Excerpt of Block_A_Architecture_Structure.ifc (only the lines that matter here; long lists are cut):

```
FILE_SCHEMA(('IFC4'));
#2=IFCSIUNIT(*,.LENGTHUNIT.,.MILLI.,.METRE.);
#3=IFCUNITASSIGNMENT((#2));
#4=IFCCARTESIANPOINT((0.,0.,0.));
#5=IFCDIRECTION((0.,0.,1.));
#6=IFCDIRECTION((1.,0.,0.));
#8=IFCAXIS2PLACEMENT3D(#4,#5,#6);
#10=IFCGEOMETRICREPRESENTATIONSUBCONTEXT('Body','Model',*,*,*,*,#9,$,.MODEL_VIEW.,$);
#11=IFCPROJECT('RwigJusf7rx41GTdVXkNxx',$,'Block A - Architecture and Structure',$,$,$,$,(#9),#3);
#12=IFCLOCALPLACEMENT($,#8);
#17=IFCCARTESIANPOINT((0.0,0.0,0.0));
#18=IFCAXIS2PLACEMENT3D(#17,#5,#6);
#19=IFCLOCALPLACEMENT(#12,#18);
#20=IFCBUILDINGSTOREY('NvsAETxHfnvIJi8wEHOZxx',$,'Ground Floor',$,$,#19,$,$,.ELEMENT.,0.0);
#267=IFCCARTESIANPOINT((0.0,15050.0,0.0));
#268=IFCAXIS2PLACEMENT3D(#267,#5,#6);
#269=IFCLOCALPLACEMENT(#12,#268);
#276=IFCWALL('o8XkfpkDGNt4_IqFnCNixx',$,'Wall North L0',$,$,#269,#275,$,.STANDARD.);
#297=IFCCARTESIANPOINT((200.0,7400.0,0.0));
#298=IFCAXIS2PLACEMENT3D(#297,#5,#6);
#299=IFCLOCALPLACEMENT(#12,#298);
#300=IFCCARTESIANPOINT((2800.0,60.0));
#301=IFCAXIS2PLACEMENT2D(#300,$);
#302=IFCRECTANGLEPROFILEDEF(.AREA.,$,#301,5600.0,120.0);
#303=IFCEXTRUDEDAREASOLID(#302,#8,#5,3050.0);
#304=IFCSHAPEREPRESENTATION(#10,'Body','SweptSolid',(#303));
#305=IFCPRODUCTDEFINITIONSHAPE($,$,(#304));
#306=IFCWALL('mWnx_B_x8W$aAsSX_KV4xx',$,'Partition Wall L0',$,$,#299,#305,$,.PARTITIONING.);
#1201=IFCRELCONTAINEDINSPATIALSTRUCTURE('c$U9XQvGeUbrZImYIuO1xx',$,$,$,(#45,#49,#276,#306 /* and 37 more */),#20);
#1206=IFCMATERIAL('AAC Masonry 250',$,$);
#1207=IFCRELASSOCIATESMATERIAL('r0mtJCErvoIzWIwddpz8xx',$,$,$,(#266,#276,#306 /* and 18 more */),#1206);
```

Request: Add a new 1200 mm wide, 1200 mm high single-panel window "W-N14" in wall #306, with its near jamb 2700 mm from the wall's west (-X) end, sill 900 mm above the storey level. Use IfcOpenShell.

```python
import numpy as np
import ifcopenshell
import ifcopenshell.api.feature
import ifcopenshell.api.geometry
import ifcopenshell.api.root
import ifcopenshell.api.spatial
import ifcopenshell.geom
import ifcopenshell.util.element
import ifcopenshell.util.placement
import ifcopenshell.util.representation
import ifcopenshell.util.shape
import ifcopenshell.util.unit

model = ifcopenshell.open("Block_A_Architecture_Structure.ifc")
unit_scale = ifcopenshell.util.unit.calculate_unit_scale(model)
settings = ifcopenshell.geom.settings()


def volume(element):
    """Net volume in cubic metres, openings subtracted."""
    shape = ifcopenshell.geom.create_shape(settings, element)
    return ifcopenshell.util.shape.get_volume(shape.geometry)


wall = model.by_guid("mWnx_B_x8W$aAsSX_KV4xx")
storey = ifcopenshell.util.element.get_container(wall, ifc_class="IfcBuildingStorey")
context = ifcopenshell.util.representation.get_context(model, "Model", "Body", "MODEL_VIEW")
before = volume(wall)

width, height, from_end, sill = 1.2, 1.2, 2.7, 0.9  # metres

# The wall runs along its own X axis, and the end named is its -X end.
wall_shape = ifcopenshell.geom.create_shape(settings, wall)
x, y, z = ifcopenshell.util.shape.get_vertices(wall_shape.geometry).T
start = x.min() + from_end
face, thickness = float(y.min()), float(y.max() - y.min())
wall_matrix = ifcopenshell.util.placement.get_local_placement(wall.ObjectPlacement)
level = ifcopenshell.util.placement.get_local_placement(storey.ObjectPlacement)[2, 3]


def in_wall(x, y):
    """Placement at x, y metres in the wall's axes, at sill height."""
    matrix = wall_matrix.copy()
    matrix[:, 3] = wall_matrix @ np.array([x / unit_scale, y / unit_scale, 0.0, 1.0])
    matrix[2, 3] = level + sill / unit_scale
    return matrix


# Opening: a box that overshoots both wall faces by 50 mm.
opening = ifcopenshell.api.root.create_entity(model, ifc_class="IfcOpeningElement", predefined_type="OPENING")
box = ifcopenshell.api.geometry.add_wall_representation(
    model, context=context, length=width, height=height, thickness=thickness + 0.1
)
ifcopenshell.api.geometry.assign_representation(model, product=opening, representation=box)
ifcopenshell.api.geometry.edit_object_placement(model, product=opening, matrix=in_wall(start, face - 0.05), is_si=False)
ifcopenshell.api.feature.add_feature(model, feature=opening, element=wall)

window = ifcopenshell.api.root.create_entity(model, ifc_class="IfcWindow", name="W-N14", predefined_type="WINDOW")
window.OverallWidth, window.OverallHeight = width / unit_scale, height / unit_scale
window.PartitioningType = "SINGLE_PANEL"
body = ifcopenshell.api.geometry.add_window_representation(
    model,
    context=context,
    overall_width=window.OverallWidth,
    overall_height=window.OverallHeight,
    partition_type="SINGLE_PANEL",
)
ifcopenshell.api.geometry.assign_representation(model, product=window, representation=body)
ifcopenshell.api.spatial.assign_container(model, products=[window], relating_structure=storey)
ifcopenshell.api.feature.add_filling(model, opening=opening, element=window)

# Centre the window in the wall's thickness.
ifcopenshell.api.geometry.edit_object_placement(model, product=window, matrix=in_wall(start, face), is_si=False)
window_shape = ifcopenshell.geom.create_shape(settings, window)
depth = ifcopenshell.util.shape.get_vertices(window_shape.geometry)[:, 1]
offset = face + thickness / 2 - (depth.min() + depth.max()) / 2
ifcopenshell.api.geometry.edit_object_placement(model, product=window, matrix=in_wall(start, offset), is_si=False)

after = volume(wall)

print(f"wall volume {before:.3f} -> {after:.3f} m3")

model.write("Block_A_Architecture_Structure_rev.ifc")
```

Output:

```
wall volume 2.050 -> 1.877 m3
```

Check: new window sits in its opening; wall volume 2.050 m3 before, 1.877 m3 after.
